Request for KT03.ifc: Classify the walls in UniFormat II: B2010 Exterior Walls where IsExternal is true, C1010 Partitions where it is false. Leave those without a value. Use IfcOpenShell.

First a look at what the model holds.

```python
import ifcopenshell
import ifcopenshell.util.element

model = ifcopenshell.open("KT03.ifc")
print(model.schema)
print("classifications:", [c.Name for c in model.by_type("IfcClassification")])
values = [ifcopenshell.util.element.get_pset(e, "Pset_WallCommon", "IsExternal") for e in model.by_type("IfcWall")]
for value in (True, False, None):
    print("IsExternal", value, values.count(value))
```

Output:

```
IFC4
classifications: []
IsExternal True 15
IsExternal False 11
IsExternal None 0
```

```python
import ifcopenshell
import ifcopenshell.api.classification
import ifcopenshell.util.element

model = ifcopenshell.open("KT03.ifc")

system = ifcopenshell.api.classification.add_classification(model, classification="UniFormat II")

walls = model.by_type("IfcWall")
external = {e: ifcopenshell.util.element.get_pset(e, "Pset_WallCommon", "IsExternal") for e in walls}
for flag, code, name in ((True, "B2010", "Exterior Walls"), (False, "C1010", "Partitions")):
    products = [e for e in walls if external[e] is flag]
    ifcopenshell.api.classification.add_reference(
        model, products=products, classification=system, identification=code, name=name
    )
    print(code, len(products))

model.write("KT03_rev.ifc")
```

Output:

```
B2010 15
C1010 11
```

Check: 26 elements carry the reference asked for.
